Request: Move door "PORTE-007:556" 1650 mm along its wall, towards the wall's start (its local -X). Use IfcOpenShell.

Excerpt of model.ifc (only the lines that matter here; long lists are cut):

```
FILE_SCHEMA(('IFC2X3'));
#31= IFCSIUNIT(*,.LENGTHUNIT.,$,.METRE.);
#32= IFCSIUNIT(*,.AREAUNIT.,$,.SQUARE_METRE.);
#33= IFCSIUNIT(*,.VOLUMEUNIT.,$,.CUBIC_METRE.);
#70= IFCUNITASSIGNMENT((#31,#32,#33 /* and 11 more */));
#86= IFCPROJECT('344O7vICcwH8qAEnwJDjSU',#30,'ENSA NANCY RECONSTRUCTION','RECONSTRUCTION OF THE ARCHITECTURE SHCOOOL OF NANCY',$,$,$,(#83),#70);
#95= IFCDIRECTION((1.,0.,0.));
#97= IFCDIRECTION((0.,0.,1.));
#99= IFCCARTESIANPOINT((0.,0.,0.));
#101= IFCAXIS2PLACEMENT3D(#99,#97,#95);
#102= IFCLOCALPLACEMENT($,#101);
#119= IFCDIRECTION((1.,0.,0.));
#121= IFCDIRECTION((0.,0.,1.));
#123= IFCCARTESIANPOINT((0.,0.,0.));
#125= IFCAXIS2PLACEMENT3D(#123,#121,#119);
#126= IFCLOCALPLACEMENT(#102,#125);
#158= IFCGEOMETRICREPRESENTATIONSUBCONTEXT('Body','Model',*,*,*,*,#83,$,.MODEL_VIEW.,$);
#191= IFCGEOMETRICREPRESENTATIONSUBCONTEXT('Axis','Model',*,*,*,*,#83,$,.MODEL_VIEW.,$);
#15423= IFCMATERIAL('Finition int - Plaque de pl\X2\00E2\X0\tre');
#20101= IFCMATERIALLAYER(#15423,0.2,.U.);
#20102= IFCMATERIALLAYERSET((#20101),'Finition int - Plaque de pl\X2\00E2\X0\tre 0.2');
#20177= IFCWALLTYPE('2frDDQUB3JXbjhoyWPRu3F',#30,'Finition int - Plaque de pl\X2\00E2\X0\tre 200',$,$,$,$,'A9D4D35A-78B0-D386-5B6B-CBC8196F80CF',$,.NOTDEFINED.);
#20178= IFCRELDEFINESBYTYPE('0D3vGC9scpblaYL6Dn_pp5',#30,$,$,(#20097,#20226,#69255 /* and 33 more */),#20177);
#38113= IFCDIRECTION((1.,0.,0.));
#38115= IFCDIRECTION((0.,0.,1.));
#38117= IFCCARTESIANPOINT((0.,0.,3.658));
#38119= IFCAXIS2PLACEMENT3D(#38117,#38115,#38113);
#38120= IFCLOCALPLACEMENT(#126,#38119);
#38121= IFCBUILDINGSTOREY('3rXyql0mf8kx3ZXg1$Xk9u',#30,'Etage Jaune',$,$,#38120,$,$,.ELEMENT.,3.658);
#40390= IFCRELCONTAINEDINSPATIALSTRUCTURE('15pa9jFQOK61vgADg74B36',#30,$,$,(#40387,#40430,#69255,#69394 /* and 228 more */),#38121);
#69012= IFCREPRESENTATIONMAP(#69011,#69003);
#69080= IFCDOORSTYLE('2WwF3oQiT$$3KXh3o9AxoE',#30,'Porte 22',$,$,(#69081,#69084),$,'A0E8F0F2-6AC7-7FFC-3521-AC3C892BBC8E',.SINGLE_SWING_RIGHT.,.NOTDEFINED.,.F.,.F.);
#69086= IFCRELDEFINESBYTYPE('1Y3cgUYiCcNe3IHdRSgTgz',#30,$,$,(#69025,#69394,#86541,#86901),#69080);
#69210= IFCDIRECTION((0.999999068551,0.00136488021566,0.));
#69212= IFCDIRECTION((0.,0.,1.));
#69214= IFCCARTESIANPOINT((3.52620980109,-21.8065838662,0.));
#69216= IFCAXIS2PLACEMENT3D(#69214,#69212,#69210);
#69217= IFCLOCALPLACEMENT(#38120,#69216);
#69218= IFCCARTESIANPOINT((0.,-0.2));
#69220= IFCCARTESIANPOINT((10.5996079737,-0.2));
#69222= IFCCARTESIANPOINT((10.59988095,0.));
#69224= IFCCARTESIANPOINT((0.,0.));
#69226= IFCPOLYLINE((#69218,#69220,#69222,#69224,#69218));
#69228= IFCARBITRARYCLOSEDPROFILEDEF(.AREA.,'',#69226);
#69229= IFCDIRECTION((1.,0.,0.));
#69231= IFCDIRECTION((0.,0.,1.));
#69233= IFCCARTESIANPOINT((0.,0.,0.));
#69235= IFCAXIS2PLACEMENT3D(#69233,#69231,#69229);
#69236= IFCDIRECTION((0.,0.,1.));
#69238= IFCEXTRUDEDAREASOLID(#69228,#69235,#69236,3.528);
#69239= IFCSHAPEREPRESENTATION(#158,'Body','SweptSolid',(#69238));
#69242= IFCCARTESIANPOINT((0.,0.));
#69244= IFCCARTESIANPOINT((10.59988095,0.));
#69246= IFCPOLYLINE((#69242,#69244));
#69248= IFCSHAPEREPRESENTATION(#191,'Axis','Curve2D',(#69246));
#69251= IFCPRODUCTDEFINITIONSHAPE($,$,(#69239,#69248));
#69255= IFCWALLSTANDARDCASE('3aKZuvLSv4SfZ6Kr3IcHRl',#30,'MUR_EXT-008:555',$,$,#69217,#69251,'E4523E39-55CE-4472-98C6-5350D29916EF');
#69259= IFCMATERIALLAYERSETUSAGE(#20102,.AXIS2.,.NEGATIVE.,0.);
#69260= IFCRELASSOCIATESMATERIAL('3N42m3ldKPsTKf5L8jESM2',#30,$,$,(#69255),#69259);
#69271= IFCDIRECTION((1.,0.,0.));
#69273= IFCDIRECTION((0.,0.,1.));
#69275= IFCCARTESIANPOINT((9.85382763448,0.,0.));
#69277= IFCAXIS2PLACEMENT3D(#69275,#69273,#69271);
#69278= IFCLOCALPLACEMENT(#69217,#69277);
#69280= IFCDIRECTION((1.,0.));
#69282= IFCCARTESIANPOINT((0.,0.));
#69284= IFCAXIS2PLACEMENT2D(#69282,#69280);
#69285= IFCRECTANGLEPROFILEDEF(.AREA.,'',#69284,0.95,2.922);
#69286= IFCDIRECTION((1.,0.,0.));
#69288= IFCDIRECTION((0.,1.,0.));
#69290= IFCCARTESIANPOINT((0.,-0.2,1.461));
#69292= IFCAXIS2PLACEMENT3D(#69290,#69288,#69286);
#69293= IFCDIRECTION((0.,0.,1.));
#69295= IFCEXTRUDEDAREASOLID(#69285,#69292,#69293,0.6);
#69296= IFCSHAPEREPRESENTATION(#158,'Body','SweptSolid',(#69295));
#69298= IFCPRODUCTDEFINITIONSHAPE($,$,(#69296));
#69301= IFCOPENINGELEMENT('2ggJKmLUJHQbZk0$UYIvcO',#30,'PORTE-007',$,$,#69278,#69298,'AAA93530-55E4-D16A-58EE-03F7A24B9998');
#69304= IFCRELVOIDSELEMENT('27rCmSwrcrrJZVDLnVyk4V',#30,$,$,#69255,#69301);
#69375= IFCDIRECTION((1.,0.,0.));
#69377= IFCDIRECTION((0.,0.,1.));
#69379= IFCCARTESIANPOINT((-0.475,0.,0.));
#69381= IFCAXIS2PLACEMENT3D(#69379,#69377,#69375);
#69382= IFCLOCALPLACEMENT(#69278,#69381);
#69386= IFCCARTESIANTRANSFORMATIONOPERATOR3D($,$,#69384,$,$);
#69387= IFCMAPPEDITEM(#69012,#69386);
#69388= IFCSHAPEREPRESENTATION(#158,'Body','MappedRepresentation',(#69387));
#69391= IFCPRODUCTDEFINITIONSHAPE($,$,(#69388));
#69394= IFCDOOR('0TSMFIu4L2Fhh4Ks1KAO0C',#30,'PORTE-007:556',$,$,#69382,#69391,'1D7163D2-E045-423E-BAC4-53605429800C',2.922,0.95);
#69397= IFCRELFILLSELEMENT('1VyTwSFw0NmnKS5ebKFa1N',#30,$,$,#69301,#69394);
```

```python
import ifcopenshell
import ifcopenshell.api.geometry
import ifcopenshell.util.placement
import ifcopenshell.util.unit

model = ifcopenshell.open("model.ifc")
unit_scale = ifcopenshell.util.unit.calculate_unit_scale(model)

door = model.by_id(69394)
opening = door.FillsVoids[0].RelatingOpeningElement
wall = opening.VoidsElements[0].RelatingBuildingElement

wall_matrix = ifcopenshell.util.placement.get_local_placement(wall.ObjectPlacement)
shift = wall_matrix[:3, 0] * -1.65 / unit_scale
before = ifcopenshell.util.placement.get_local_placement(door.ObjectPlacement)[:3, 3].copy()

# The door is placed relative to its opening, so it follows when the opening moves.
matrix = ifcopenshell.util.placement.get_local_placement(opening.ObjectPlacement)
matrix[:3, 3] += shift
ifcopenshell.api.geometry.edit_object_placement(
    model, product=opening, matrix=matrix, is_si=False, should_transform_children=True
)

after = ifcopenshell.util.placement.get_local_placement(door.ObjectPlacement)[:3, 3]
print("door moved by", (after - before).round(3) + 0.0)

model.write("model_updated.ifc")
```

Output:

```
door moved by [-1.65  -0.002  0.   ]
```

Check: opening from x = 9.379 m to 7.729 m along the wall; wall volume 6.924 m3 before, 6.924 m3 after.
